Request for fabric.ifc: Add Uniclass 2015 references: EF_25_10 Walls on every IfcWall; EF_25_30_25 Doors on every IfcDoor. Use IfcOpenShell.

First a look at what the model holds.

```python
import ifcopenshell

model = ifcopenshell.open("fabric.ifc")
print(model.schema)
print("classifications:", [c.Name for c in model.by_type("IfcClassification")])
for ifc_class in ("IfcDoor", "IfcRoof", "IfcStair", "IfcWall", "IfcWindow"):
    print(ifc_class, len(model.by_type(ifc_class)))
```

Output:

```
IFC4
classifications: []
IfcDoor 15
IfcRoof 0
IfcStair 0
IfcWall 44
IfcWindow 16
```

```python
import ifcopenshell
import ifcopenshell.api.classification

model = ifcopenshell.open("fabric.ifc")

system = ifcopenshell.api.classification.add_classification(model, classification="Uniclass 2015")

codes = {
    "IfcWall": ("EF_25_10", "Walls"),
    "IfcDoor": ("EF_25_30_25", "Doors"),
}
for ifc_class, (code, name) in codes.items():
    products = model.by_type(ifc_class)
    ifcopenshell.api.classification.add_reference(
        model, products=products, classification=system, identification=code, name=name
    )
    print(code, len(products))

model.write("fabric_updated.ifc")
```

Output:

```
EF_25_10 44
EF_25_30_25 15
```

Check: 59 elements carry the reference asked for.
